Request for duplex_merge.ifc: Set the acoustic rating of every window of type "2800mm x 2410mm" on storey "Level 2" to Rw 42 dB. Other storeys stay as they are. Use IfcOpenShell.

First a look at what the model holds.

```python
import ifcopenshell
import ifcopenshell.util.element

model = ifcopenshell.open("duplex_merge.ifc")
print(model.schema)
storey = next(s for s in model.by_type("IfcBuildingStorey") if s.Name == "Level 2")
windows = [e for e in ifcopenshell.util.element.get_decomposition(storey) if e.is_a("IfcWindow")]
seen = {}
for e in windows:
    element_type = ifcopenshell.util.element.get_type(e)
    key = (element_type.Name if element_type != e and element_type else None, ifcopenshell.util.element.get_pset(e, "Pset_WindowCommon", "AcousticRating"))
    seen[key] = seen.get(key, 0) + 1
for (name, value), count in sorted(seen.items(), key=str):
    print(count, "x", name, "|", value)
```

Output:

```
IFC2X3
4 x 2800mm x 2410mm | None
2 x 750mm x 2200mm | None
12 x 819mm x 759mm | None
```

```python
import ifcopenshell
import ifcopenshell.api.pset
import ifcopenshell.util.element

model = ifcopenshell.open("duplex_merge.ifc")

storey = next(s for s in model.by_type("IfcBuildingStorey") if s.Name == "Level 2")
windows = [e for e in ifcopenshell.util.element.get_decomposition(storey) if e.is_a("IfcWindow")]

count = 0
for e in windows:
    element_type = ifcopenshell.util.element.get_type(e)
    if element_type in (None, e) or element_type.Name != "2800mm x 2410mm":
        continue
    # add_pset returns the element's existing set when there is one.
    pset = ifcopenshell.api.pset.add_pset(model, product=e, name="Pset_WindowCommon")
    ifcopenshell.api.pset.edit_pset(model, pset=pset, properties={"AcousticRating": "Rw 42 dB"})
    count += 1

print(count, "windows updated")

model.write("duplex_merge_updated.ifc")
```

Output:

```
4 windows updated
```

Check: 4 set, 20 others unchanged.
